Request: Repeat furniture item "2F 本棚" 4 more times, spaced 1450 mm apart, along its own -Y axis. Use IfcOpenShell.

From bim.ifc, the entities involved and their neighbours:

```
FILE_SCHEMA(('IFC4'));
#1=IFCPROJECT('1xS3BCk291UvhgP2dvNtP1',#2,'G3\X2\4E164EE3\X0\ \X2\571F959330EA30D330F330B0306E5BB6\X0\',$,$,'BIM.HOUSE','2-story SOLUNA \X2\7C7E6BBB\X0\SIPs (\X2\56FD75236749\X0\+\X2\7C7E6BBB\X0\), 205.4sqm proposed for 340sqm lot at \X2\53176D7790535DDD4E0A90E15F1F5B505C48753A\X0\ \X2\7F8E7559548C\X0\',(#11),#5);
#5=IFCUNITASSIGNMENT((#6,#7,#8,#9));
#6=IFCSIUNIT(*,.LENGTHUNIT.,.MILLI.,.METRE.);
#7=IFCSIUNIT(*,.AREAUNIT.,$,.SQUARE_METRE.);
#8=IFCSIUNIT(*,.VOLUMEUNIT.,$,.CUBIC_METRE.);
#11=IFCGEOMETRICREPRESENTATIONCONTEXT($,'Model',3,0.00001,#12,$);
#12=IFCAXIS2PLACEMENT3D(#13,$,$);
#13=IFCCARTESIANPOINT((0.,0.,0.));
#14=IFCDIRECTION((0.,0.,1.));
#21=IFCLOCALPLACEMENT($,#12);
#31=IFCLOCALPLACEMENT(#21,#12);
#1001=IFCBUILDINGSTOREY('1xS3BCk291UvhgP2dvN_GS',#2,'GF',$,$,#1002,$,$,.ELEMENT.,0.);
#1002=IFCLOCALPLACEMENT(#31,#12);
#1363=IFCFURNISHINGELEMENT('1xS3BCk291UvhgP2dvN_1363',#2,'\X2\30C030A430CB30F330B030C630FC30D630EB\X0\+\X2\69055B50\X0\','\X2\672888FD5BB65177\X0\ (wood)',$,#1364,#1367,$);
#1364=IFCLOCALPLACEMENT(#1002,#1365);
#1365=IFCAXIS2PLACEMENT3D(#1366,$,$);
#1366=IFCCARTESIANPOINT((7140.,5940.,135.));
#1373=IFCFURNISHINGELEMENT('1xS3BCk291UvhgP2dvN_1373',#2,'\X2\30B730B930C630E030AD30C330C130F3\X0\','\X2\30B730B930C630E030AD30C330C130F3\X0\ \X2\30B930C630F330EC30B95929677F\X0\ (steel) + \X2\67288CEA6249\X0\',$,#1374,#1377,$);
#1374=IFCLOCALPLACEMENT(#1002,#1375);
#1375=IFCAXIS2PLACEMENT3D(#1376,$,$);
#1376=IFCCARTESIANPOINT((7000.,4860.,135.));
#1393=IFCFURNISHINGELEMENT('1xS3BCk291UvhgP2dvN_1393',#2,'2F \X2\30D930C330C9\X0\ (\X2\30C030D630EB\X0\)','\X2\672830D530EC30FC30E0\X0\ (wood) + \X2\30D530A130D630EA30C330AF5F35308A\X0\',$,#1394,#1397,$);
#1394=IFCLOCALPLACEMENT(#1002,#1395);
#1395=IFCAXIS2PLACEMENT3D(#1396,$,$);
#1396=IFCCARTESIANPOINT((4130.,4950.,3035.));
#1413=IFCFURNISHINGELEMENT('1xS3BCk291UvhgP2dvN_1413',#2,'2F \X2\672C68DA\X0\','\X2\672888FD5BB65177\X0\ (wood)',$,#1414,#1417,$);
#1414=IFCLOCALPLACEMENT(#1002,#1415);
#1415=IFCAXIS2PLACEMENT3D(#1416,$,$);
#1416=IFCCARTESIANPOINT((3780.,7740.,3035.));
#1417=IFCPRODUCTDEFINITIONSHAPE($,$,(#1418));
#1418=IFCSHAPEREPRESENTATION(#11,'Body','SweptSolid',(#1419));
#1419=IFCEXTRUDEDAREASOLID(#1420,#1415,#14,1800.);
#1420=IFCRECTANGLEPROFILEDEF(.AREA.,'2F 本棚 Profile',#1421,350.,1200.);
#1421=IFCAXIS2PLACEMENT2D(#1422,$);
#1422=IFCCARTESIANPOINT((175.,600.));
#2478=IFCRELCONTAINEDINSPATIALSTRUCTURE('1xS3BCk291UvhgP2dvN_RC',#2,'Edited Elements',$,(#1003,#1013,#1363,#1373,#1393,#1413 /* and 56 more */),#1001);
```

```python
import ifcopenshell
import ifcopenshell.api.geometry
import ifcopenshell.api.root
import ifcopenshell.util.element
import ifcopenshell.util.placement
import ifcopenshell.util.unit

model = ifcopenshell.open("bim.ifc")
unit_scale = ifcopenshell.util.unit.calculate_unit_scale(model)


def reuse_history(source, copy):
    """copy_class also copies each property set's owner history, people and application; keep the originals."""
    for rel in copy.IsDefinedBy:
        if rel.is_a("IfcRelDefinesByProperties") and (history := rel.RelatingPropertyDefinition.OwnerHistory):
            rel.RelatingPropertyDefinition.OwnerHistory = source.OwnerHistory
            ifcopenshell.util.element.remove_deep2(model, history)


source = model.by_guid("1xS3BCk291UvhgP2dvN_1413")
base = ifcopenshell.util.placement.get_local_placement(source.ObjectPlacement)
step = -base[:3, 1] * 1.45 / unit_scale

for i in range(1, 5):
    copy = ifcopenshell.api.root.copy_class(model, product=source)
    copy.Representation = ifcopenshell.util.element.copy_deep(
        model, source.Representation, exclude=["IfcGeometricRepresentationContext", "IfcRepresentationMap"]
    )
    reuse_history(source, copy)
    matrix = base.copy()
    matrix[:3, 3] += i * step
    print("added at", matrix[:3, 3].round(3) + 0.0)
    ifcopenshell.api.geometry.edit_object_placement(model, product=copy, matrix=matrix, is_si=False)

model.write("bim_v2.ifc")
```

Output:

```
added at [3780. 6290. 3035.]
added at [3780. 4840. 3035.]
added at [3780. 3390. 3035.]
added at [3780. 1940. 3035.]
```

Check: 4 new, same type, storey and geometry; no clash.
